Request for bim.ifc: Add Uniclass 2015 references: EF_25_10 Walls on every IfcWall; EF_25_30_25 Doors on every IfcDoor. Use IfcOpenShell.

First a look at what the model holds.

```python
import ifcopenshell

model = ifcopenshell.open("bim.ifc")
print(model.schema)
print("classifications:", [c.Name for c in model.by_type("IfcClassification")])
for ifc_class in ("IfcDoor", "IfcRoof", "IfcStair", "IfcWall", "IfcWindow"):
    print(ifc_class, len(model.by_type(ifc_class)))
```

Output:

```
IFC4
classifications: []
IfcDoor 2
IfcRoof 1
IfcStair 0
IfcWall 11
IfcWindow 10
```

```python
import ifcopenshell
import ifcopenshell.api.classification

model = ifcopenshell.open("bim.ifc")

system = ifcopenshell.api.classification.add_classification(model, classification="Uniclass 2015")

codes = {
    "IfcWall": ("EF_25_10", "Walls"),
    "IfcDoor": ("EF_25_30_25", "Doors"),
}
for ifc_class, (code, name) in codes.items():
    products = model.by_type(ifc_class)
    ifcopenshell.api.classification.add_reference(
        model, products=products, classification=system, identification=code, name=name
    )
    print(code, len(products))

model.write("bim_updated.ifc")
```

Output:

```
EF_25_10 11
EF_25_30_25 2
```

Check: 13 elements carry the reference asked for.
